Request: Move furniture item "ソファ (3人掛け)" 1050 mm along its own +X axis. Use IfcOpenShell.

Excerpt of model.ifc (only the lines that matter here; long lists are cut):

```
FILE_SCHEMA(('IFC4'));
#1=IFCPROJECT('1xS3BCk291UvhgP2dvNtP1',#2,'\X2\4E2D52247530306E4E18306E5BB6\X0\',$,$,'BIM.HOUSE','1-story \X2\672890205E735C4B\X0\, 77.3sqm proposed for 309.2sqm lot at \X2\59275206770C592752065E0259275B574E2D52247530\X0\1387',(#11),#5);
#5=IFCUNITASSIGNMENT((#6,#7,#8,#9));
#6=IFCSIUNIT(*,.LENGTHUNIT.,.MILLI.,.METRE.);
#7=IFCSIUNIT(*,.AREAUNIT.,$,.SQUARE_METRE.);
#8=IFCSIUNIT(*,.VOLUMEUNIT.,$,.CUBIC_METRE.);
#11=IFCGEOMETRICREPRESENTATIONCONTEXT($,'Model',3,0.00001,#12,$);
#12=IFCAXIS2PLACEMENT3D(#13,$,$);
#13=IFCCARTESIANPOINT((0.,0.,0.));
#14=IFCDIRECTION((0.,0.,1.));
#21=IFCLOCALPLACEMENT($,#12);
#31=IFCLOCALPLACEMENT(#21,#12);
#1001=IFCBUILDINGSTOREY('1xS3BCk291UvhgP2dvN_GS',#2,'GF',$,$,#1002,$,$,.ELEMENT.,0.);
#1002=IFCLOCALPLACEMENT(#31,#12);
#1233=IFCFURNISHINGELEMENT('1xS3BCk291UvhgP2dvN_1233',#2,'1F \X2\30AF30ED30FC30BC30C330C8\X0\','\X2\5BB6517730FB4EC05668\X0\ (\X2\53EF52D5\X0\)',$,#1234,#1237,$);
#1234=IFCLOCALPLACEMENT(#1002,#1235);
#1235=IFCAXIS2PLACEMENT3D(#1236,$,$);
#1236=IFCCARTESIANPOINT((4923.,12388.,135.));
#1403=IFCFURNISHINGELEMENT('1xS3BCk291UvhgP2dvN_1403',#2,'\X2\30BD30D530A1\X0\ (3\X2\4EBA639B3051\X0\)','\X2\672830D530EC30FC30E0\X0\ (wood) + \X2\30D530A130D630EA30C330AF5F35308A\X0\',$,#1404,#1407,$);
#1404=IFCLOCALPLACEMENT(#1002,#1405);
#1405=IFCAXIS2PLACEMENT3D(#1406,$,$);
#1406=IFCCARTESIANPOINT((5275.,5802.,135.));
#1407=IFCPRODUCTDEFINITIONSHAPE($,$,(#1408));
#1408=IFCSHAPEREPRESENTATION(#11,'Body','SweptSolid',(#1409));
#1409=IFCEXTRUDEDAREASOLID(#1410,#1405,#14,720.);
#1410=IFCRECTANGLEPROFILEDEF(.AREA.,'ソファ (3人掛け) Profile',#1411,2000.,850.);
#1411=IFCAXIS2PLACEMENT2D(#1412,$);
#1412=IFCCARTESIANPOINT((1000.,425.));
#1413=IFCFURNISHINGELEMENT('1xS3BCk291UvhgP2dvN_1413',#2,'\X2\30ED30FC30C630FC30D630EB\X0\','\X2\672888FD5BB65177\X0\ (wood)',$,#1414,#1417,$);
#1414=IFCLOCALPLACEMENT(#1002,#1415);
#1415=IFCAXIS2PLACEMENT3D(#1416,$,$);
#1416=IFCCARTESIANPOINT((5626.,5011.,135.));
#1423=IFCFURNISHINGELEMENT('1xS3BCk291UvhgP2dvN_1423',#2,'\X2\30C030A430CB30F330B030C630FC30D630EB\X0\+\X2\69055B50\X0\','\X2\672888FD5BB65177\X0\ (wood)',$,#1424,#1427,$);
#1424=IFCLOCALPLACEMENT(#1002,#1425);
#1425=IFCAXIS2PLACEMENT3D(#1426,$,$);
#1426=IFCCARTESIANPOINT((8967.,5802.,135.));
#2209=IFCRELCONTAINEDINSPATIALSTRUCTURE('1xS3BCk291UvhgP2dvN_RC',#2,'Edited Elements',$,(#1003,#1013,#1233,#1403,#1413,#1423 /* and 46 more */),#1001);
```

```python
import ifcopenshell
import ifcopenshell.api.geometry
import ifcopenshell.util.placement
import ifcopenshell.util.unit

model = ifcopenshell.open("model.ifc")
unit_scale = ifcopenshell.util.unit.calculate_unit_scale(model)

item = model.by_id(1403)
matrix = ifcopenshell.util.placement.get_local_placement(item.ObjectPlacement)
matrix[:3, 3] += matrix[:3, 0] * 1.05 / unit_scale
ifcopenshell.api.geometry.edit_object_placement(model, product=item, matrix=matrix, is_si=False)

print(ifcopenshell.util.placement.get_local_placement(item.ObjectPlacement).round(3) + 0.0)

model.write("model_rev.ifc")
```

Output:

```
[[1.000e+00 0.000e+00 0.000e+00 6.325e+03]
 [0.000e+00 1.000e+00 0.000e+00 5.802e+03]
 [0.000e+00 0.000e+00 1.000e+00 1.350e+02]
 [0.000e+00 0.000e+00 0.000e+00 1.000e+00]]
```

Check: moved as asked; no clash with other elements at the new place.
